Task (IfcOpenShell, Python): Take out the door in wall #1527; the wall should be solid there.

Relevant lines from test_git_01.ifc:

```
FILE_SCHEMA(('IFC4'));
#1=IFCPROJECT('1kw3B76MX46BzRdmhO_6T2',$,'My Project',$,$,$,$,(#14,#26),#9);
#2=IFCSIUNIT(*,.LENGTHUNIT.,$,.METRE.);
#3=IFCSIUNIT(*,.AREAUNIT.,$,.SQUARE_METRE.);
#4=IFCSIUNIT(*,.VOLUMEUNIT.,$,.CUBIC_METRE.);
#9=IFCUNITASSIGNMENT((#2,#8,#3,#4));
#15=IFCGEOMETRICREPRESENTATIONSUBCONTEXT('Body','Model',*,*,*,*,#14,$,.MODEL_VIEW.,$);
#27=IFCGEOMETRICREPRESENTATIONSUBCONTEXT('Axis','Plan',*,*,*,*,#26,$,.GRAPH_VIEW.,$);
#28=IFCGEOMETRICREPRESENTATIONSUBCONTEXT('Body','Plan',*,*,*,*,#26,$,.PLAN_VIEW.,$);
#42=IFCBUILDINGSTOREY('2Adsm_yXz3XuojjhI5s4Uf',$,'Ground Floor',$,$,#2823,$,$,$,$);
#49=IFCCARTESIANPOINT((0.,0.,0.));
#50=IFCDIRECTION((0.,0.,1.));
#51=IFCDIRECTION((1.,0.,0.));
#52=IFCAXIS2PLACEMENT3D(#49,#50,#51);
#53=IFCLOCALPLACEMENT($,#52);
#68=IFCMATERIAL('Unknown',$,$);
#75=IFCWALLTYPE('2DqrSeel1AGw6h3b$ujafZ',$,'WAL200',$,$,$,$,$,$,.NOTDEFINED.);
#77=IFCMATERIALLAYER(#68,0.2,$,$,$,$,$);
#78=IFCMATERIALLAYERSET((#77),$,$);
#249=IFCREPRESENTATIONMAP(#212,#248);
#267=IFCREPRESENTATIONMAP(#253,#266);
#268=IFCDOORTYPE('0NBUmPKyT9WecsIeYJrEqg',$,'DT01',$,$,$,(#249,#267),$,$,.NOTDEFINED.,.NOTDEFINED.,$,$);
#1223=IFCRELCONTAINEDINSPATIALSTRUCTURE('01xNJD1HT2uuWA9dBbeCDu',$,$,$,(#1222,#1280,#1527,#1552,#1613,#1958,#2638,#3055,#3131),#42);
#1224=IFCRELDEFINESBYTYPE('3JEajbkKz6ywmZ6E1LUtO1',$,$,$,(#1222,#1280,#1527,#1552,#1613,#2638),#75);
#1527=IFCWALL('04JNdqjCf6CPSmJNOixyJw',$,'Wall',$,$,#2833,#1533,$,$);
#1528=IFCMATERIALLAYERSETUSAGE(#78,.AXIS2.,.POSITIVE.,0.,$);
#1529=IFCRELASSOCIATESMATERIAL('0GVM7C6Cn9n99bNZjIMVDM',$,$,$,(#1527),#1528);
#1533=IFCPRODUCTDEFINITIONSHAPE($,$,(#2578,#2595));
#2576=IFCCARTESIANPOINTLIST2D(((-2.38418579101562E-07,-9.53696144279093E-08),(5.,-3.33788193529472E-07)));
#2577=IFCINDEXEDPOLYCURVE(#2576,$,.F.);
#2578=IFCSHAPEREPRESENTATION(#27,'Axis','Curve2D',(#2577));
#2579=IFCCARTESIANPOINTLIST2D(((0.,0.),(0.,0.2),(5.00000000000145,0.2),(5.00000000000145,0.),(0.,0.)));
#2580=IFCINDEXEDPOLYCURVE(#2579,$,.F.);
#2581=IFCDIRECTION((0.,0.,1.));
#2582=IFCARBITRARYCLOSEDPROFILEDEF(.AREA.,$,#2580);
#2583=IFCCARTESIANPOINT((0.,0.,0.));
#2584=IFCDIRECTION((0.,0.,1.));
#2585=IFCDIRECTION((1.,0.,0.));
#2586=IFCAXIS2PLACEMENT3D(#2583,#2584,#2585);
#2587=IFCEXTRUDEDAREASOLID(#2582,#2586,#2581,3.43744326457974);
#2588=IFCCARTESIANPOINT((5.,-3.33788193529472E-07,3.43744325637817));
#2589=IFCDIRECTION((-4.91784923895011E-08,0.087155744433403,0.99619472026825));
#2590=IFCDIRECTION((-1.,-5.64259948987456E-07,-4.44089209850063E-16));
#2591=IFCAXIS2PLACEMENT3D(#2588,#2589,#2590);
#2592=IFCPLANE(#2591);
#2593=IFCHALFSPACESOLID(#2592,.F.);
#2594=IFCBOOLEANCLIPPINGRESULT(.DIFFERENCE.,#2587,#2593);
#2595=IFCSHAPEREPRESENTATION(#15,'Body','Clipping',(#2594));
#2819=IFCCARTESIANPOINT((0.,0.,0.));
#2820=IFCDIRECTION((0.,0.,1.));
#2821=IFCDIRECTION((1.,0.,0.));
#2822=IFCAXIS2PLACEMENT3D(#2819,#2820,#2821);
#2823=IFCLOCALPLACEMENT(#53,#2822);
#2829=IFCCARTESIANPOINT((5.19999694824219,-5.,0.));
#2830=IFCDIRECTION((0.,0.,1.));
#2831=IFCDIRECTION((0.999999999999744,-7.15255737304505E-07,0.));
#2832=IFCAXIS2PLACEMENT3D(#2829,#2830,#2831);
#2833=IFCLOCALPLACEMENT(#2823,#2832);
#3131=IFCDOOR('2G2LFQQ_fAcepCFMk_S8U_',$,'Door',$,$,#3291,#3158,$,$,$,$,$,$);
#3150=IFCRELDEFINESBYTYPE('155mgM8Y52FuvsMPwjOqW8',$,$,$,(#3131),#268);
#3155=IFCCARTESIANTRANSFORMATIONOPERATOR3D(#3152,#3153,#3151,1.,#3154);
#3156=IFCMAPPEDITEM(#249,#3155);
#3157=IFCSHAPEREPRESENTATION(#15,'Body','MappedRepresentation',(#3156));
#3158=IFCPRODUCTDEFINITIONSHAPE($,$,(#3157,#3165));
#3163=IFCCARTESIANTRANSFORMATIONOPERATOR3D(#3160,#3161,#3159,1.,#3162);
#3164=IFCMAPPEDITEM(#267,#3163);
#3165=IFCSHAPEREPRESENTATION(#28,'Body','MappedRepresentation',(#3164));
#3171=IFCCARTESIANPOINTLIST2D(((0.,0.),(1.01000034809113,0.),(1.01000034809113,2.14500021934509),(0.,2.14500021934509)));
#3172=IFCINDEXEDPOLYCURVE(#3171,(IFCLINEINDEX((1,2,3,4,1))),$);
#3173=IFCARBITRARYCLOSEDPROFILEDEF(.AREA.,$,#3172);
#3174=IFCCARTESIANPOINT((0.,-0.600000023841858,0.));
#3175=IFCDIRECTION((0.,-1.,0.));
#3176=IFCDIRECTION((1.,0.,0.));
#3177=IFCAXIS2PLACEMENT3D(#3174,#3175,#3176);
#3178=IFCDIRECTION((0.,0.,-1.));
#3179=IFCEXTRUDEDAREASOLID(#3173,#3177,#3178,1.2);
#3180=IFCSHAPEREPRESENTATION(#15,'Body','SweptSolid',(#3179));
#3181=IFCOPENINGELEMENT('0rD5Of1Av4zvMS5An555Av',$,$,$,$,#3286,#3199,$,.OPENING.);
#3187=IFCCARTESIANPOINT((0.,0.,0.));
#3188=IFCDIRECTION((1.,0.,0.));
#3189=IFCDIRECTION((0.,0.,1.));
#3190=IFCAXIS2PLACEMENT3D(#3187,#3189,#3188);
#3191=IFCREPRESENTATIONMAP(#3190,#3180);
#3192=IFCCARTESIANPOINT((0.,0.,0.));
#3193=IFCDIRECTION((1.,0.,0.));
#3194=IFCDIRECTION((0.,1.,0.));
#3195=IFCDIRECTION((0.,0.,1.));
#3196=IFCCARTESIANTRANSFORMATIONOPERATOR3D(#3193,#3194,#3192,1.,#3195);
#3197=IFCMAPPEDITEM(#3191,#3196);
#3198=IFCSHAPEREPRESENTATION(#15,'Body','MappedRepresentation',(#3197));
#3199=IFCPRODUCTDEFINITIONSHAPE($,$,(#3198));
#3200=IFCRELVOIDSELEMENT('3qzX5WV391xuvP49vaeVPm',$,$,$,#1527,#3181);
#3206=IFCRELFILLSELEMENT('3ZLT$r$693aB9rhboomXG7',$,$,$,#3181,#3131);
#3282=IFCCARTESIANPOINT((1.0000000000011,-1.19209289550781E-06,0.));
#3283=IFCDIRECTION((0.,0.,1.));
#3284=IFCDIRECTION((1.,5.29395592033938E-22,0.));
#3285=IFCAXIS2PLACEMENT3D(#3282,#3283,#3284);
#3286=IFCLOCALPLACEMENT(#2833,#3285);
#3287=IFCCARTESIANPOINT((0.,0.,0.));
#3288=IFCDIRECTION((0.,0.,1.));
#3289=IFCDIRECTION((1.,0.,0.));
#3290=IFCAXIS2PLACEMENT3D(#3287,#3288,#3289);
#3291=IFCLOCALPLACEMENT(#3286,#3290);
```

```python
import ifcopenshell
import ifcopenshell.api.feature
import ifcopenshell.api.root
import ifcopenshell.geom
import ifcopenshell.util.shape

model = ifcopenshell.open("test_git_01.ifc")
settings = ifcopenshell.geom.settings()


def volume(element):
    """Net volume in cubic metres, openings subtracted."""
    shape = ifcopenshell.geom.create_shape(settings, element)
    return ifcopenshell.util.shape.get_volume(shape.geometry)


door = model.by_guid("2G2LFQQ_fAcepCFMk_S8U_")
opening = door.FillsVoids[0].RelatingOpeningElement
wall = opening.VoidsElements[0].RelatingBuildingElement
before = volume(wall)

ifcopenshell.api.root.remove_product(model, product=door)
ifcopenshell.api.feature.remove_feature(model, feature=opening)

after = volume(wall)

print(f"wall volume {before:.3f} -> {after:.3f} m3")

model.write("test_git_01_v2.ifc")
```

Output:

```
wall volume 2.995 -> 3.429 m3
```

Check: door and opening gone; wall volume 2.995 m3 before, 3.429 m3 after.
